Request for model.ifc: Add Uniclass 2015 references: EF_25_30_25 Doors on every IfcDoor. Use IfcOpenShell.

First a look at what the model holds.

```python
import ifcopenshell

model = ifcopenshell.open("model.ifc")
print(model.schema)
print("classifications:", [c.Name for c in model.by_type("IfcClassification")])
for ifc_class in ("IfcDoor", "IfcRoof", "IfcStair", "IfcWall", "IfcWindow"):
    print(ifc_class, len(model.by_type(ifc_class)))
```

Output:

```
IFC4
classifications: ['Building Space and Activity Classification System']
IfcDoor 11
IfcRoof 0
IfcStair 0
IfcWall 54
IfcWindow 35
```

```python
import ifcopenshell
import ifcopenshell.api.classification

model = ifcopenshell.open("model.ifc")

system = ifcopenshell.api.classification.add_classification(model, classification="Uniclass 2015")

codes = {
    "IfcDoor": ("EF_25_30_25", "Doors"),
}
for ifc_class, (code, name) in codes.items():
    products = model.by_type(ifc_class)
    ifcopenshell.api.classification.add_reference(
        model, products=products, classification=system, identification=code, name=name
    )
    print(code, len(products))

model.write("model_rev.ifc")
```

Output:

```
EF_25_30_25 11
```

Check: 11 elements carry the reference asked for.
